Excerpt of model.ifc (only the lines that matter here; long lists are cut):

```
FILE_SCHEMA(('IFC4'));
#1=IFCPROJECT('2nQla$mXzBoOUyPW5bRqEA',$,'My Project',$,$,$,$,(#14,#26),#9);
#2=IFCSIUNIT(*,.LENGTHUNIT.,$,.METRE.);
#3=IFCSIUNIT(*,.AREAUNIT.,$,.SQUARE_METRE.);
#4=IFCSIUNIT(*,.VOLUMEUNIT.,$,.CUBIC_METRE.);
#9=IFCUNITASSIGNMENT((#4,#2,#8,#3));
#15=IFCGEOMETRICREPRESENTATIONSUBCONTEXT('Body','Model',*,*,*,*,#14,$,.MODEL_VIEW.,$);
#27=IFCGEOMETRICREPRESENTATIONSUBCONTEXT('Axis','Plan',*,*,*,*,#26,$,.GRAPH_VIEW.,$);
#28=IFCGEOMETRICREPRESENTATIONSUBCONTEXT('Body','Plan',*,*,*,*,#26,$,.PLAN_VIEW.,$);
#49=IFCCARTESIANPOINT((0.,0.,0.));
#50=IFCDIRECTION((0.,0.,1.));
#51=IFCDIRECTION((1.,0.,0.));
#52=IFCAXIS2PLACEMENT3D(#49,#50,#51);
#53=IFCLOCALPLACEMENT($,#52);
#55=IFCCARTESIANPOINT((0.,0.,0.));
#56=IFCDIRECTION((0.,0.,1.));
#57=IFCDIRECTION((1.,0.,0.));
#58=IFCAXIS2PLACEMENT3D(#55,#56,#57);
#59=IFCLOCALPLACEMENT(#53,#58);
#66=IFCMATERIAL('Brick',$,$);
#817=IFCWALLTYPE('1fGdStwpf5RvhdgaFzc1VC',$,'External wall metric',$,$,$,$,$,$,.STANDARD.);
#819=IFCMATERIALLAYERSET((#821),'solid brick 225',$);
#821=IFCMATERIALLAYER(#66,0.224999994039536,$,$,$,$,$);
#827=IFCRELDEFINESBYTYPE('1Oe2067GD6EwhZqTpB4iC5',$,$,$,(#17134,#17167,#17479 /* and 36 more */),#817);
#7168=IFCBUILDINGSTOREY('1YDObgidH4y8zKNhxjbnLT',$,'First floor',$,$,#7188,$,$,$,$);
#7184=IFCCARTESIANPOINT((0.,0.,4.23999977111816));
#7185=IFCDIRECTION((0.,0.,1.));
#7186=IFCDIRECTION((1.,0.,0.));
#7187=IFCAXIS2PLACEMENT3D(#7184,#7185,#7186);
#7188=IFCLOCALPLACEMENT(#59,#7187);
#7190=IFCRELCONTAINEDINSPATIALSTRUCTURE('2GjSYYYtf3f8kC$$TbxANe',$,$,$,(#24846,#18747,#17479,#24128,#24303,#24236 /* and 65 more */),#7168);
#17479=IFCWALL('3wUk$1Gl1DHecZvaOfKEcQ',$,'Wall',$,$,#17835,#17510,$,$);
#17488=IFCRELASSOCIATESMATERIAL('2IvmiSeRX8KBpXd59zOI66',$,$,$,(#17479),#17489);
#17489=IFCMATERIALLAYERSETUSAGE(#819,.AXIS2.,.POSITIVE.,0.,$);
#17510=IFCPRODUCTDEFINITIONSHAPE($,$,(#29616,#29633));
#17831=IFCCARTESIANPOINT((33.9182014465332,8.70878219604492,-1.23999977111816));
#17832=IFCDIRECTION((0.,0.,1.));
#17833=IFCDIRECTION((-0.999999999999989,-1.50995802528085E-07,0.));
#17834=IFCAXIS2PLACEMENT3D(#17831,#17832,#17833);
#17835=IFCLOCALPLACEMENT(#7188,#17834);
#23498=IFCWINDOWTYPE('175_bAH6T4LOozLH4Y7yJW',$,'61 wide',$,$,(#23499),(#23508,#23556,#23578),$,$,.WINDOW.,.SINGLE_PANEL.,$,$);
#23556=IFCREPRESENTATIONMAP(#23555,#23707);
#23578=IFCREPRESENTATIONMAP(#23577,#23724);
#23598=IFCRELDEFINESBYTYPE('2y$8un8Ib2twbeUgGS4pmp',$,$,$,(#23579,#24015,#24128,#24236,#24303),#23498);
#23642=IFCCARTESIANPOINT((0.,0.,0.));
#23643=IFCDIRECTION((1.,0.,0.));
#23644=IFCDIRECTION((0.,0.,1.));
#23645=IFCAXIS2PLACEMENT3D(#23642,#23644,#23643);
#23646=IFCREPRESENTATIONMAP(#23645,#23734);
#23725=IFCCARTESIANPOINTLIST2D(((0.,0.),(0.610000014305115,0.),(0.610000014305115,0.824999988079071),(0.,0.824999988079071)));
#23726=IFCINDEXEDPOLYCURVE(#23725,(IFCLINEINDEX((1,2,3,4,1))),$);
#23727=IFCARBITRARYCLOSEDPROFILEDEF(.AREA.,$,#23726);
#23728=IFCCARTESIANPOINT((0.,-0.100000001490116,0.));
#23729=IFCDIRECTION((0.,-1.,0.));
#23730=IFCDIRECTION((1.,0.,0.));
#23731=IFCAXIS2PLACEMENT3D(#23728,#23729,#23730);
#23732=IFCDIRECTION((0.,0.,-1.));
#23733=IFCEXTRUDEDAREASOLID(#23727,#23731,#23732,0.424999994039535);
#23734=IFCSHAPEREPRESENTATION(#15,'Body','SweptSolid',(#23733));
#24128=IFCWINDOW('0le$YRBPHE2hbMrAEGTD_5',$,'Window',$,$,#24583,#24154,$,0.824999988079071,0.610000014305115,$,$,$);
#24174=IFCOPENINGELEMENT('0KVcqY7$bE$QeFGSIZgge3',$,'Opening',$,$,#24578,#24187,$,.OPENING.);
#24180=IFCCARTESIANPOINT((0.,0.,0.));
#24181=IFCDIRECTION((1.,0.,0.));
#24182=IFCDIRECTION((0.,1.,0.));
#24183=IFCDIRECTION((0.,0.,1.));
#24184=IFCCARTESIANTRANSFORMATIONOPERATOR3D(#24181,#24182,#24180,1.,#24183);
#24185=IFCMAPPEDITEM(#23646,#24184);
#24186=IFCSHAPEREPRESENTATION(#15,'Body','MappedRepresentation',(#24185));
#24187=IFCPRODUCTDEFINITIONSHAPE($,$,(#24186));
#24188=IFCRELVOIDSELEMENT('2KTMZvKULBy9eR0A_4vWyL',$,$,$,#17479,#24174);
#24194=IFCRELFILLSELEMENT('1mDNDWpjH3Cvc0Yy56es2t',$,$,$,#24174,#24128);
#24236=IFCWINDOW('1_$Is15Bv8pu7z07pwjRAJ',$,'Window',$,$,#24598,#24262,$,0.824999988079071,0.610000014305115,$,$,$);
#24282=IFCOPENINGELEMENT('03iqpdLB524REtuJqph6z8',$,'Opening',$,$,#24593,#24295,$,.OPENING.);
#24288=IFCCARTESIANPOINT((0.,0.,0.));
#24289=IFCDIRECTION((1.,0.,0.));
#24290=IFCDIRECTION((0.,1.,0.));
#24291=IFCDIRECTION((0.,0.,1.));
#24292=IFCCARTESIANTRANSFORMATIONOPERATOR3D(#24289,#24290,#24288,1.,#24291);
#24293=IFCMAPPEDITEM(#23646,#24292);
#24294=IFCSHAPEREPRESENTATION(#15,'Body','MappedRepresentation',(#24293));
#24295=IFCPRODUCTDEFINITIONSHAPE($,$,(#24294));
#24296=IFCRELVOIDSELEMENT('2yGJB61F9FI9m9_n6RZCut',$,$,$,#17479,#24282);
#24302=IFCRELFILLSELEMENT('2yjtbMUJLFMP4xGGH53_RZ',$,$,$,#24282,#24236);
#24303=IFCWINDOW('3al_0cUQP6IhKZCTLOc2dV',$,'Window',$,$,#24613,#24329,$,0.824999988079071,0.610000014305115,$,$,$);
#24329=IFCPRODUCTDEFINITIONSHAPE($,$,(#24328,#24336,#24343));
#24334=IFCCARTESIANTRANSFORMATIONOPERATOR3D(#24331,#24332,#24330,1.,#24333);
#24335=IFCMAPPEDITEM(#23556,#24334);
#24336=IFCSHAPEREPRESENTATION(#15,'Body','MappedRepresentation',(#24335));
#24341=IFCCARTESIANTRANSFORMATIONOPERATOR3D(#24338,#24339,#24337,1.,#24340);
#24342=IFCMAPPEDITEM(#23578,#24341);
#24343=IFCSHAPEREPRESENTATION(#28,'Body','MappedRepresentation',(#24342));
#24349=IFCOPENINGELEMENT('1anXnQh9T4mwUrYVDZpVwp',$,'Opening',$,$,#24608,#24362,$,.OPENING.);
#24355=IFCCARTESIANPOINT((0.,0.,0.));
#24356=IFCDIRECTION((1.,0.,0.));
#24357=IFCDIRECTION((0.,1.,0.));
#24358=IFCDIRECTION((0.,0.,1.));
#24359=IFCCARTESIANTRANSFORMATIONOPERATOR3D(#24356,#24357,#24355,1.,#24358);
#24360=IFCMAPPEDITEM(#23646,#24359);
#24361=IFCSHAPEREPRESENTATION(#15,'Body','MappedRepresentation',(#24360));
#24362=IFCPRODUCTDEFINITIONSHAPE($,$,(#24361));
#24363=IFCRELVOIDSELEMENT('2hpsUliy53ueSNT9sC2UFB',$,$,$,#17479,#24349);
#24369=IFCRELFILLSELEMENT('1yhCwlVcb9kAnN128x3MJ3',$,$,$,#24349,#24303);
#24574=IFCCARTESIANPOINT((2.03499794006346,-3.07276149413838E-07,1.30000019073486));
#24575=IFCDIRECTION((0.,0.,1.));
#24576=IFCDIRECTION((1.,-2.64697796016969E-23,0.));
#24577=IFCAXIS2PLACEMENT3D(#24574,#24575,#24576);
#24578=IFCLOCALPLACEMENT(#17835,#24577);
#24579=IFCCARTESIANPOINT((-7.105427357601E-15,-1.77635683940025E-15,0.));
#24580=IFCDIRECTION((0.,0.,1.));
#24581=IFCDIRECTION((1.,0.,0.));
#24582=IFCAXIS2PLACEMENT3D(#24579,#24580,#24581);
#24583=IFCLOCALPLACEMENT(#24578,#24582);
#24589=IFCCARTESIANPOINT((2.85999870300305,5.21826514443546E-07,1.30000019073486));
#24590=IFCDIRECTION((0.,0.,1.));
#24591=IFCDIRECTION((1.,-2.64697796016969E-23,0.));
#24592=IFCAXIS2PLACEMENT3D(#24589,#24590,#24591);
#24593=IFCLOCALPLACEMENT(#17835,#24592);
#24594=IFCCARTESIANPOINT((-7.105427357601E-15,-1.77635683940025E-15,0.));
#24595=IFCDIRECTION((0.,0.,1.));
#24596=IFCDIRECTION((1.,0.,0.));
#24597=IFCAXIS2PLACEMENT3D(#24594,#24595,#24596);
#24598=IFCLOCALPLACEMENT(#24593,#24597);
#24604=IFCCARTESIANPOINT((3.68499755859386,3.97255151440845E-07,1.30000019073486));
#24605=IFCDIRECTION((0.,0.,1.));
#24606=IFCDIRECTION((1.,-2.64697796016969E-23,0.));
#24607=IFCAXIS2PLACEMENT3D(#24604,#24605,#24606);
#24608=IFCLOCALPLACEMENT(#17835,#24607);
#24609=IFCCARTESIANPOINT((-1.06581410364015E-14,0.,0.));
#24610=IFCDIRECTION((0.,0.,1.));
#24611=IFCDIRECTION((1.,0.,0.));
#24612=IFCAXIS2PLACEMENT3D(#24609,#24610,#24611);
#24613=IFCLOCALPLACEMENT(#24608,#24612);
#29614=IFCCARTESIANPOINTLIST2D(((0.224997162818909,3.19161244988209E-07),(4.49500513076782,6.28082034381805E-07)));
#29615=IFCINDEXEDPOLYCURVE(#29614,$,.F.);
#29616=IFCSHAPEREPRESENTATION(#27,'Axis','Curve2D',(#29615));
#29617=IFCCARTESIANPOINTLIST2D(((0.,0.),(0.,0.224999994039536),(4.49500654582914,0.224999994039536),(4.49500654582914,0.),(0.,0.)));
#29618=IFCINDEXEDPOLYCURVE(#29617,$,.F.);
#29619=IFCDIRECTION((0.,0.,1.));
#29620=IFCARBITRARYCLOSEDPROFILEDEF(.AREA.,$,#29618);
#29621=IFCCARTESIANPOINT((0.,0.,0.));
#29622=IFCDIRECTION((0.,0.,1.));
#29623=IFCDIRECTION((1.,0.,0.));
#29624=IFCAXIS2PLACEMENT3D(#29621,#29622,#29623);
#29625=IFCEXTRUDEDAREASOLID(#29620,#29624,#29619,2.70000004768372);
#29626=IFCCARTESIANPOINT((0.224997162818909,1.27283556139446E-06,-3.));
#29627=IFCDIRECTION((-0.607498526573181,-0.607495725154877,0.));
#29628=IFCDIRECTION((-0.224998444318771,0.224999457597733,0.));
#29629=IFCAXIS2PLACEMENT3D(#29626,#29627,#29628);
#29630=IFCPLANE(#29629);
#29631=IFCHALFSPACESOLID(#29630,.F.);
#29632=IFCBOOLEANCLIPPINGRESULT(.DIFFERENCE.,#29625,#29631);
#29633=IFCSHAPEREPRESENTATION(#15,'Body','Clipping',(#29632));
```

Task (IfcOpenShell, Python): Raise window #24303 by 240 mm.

```python
import numpy as np
import ifcopenshell
import ifcopenshell.api.geometry
import ifcopenshell.util.placement
import ifcopenshell.util.unit

model = ifcopenshell.open("model.ifc")
unit_scale = ifcopenshell.util.unit.calculate_unit_scale(model)

window = model.by_id(24303)
opening = window.FillsVoids[0].RelatingOpeningElement
dz = 0.24

shift = np.array([0.0, 0.0, dz])
# The window is placed relative to its opening, so it follows when the opening moves.
matrix = ifcopenshell.util.placement.get_local_placement(opening.ObjectPlacement)
matrix[:3, 3] += shift
ifcopenshell.api.geometry.edit_object_placement(
    model, product=opening, matrix=matrix, is_si=False, should_transform_children=True
)

print(f"moved by {dz * unit_scale:+.3f} m")

model.write("model_v2.ifc")
```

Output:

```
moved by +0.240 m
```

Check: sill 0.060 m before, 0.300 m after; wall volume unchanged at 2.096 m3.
